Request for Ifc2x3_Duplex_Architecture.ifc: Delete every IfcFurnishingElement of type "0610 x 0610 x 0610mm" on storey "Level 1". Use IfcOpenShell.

First a look at what the model holds.

```python
import ifcopenshell
import ifcopenshell.util.element

model = ifcopenshell.open("Ifc2x3_Duplex_Architecture.ifc")
print(model.schema)
storey = next(s for s in model.by_type("IfcBuildingStorey") if s.Name == "Level 1")
furniture = [e for e in ifcopenshell.util.element.get_decomposition(storey) if e.is_a("IfcFurnishingElement")]
seen = {}
for e in furniture:
    element_type = ifcopenshell.util.element.get_type(e)
    name = element_type.Name if element_type not in (None, e) else None
    seen[name] = seen.get(name, 0) + 1
for name, count in sorted(seen.items(), key=str):
    print(count, "x", name)
```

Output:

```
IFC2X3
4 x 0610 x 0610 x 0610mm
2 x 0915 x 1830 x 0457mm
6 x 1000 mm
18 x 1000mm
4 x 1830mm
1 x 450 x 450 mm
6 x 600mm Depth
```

```python
import ifcopenshell
import ifcopenshell.api.root
import ifcopenshell.util.element

model = ifcopenshell.open("Ifc2x3_Duplex_Architecture.ifc")

storey = next(s for s in model.by_type("IfcBuildingStorey") if s.Name == "Level 1")
furniture = [e for e in ifcopenshell.util.element.get_decomposition(storey) if e.is_a("IfcFurnishingElement")]
targets = [e for e in furniture if (t := ifcopenshell.util.element.get_type(e)) not in (None, e) and t.Name == "0610 x 0610 x 0610mm"]

for e in targets:
    ifcopenshell.api.root.remove_product(model, product=e)
print(len(targets), "removed")

model.write("Ifc2x3_Duplex_Architecture_updated.ifc")
```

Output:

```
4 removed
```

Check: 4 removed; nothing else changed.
